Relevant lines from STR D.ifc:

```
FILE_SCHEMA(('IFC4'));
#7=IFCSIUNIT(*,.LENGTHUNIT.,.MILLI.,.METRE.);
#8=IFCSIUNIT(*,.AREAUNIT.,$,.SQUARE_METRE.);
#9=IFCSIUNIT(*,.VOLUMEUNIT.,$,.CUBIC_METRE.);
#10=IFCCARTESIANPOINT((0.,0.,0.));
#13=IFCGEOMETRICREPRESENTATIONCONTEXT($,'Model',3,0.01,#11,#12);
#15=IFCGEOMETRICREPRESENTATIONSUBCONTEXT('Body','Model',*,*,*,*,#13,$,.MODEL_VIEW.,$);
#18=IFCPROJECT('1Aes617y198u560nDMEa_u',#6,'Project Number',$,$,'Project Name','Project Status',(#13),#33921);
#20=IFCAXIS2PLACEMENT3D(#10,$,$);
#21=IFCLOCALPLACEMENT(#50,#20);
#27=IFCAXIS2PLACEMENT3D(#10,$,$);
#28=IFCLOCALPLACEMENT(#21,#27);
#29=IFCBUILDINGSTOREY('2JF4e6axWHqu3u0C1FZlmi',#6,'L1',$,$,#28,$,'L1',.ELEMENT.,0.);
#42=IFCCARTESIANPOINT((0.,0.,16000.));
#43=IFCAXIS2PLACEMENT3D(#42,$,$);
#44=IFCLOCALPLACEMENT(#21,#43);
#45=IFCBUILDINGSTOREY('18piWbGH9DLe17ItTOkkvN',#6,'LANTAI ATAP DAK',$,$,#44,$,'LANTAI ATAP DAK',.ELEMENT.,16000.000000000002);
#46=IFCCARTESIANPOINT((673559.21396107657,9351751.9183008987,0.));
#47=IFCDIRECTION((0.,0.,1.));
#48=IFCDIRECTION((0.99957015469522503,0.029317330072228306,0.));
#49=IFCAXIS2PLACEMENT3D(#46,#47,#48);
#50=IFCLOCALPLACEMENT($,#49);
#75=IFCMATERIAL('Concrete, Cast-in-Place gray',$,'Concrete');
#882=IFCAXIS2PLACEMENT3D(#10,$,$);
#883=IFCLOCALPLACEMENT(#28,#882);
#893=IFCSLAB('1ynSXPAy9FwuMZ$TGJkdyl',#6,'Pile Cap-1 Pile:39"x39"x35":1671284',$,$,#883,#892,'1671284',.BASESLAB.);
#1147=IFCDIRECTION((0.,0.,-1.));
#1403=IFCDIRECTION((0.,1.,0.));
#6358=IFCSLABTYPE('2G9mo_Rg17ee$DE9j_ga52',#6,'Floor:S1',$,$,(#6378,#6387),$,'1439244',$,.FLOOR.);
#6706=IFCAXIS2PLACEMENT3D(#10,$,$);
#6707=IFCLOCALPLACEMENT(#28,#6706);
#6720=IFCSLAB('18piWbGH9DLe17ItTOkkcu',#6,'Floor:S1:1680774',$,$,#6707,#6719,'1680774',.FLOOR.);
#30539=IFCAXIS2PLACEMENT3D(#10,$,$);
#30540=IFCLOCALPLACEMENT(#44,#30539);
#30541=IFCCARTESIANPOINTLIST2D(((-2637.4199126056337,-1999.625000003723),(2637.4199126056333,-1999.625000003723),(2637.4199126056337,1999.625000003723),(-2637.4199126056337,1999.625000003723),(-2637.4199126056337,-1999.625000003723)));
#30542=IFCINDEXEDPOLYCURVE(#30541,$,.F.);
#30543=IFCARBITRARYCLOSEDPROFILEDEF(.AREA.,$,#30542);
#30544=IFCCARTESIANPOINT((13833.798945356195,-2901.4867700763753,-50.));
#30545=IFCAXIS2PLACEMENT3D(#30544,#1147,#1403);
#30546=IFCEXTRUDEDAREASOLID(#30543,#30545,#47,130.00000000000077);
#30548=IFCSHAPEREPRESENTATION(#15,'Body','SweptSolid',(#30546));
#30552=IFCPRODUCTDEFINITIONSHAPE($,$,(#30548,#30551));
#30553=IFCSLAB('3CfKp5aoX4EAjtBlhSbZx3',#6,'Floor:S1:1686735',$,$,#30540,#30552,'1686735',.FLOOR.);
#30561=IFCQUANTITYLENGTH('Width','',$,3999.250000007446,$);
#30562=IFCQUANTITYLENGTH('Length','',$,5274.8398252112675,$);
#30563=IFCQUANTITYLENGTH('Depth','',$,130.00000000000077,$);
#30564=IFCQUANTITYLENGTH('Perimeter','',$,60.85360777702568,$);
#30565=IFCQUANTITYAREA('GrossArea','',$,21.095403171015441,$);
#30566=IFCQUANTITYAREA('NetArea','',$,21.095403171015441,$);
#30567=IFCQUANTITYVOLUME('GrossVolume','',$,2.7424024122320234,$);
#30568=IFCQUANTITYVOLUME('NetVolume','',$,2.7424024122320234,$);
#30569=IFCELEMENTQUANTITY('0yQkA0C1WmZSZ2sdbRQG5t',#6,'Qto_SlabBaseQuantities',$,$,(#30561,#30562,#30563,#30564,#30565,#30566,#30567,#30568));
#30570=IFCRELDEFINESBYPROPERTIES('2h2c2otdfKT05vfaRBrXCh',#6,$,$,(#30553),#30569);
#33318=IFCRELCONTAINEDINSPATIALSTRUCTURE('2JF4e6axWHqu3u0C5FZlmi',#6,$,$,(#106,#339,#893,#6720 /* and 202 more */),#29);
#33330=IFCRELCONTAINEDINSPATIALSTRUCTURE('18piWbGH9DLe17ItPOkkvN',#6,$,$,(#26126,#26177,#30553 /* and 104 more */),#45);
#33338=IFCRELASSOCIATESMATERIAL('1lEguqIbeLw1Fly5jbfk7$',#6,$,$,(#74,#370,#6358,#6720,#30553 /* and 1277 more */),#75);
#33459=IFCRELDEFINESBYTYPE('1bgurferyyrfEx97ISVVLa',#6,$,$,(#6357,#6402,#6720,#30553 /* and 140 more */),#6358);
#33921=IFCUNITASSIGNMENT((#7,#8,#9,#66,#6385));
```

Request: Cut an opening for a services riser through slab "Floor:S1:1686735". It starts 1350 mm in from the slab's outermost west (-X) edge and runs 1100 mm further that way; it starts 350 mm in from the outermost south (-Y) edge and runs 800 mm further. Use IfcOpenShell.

```python
import numpy as np
import ifcopenshell
import ifcopenshell.api.feature
import ifcopenshell.api.geometry
import ifcopenshell.api.pset
import ifcopenshell.api.root
import ifcopenshell.geom
import ifcopenshell.util.element
import ifcopenshell.util.placement
import ifcopenshell.util.representation
import ifcopenshell.util.shape
import ifcopenshell.util.unit

model = ifcopenshell.open("STR D.ifc")
unit_scale = ifcopenshell.util.unit.calculate_unit_scale(model)
area_scale = ifcopenshell.util.unit.calculate_unit_scale(model, "AREAUNIT")
volume_scale = ifcopenshell.util.unit.calculate_unit_scale(model, "VOLUMEUNIT")
settings = ifcopenshell.geom.settings()


def volume(element):
    """Net volume in cubic metres, openings subtracted."""
    shape = ifcopenshell.geom.create_shape(settings, element)
    return ifcopenshell.util.shape.get_volume(shape.geometry)


slab = model.by_guid("3CfKp5aoX4EAjtBlhSbZx3")
before = volume(slab)

# Extent in the slab's own axes, in metres. The edges named are its -X and -Y sides.
slab_shape = ifcopenshell.geom.create_shape(settings, slab)
vertices = ifcopenshell.util.shape.get_vertices(slab_shape.geometry)
x_min, y_min, bottom = vertices.min(axis=0)
top = vertices[:, 2].max()

opening = ifcopenshell.api.root.create_entity(model, ifc_class="IfcOpeningElement", name="Services riser opening", predefined_type="OPENING")
context = ifcopenshell.util.representation.get_context(model, "Model", "Body", "MODEL_VIEW")
width, depth = 1.1, 0.8
outline = [(0.0, 0.0), (width, 0.0), (width, depth), (0.0, depth), (0.0, 0.0)]
# Overshoot both faces by 50 mm so the cut is clean.
shape = ifcopenshell.api.geometry.add_slab_representation(
    model, context=context, depth=top - bottom + 0.1, polyline=outline
)
ifcopenshell.api.geometry.assign_representation(model, product=opening, representation=shape)

matrix = ifcopenshell.util.placement.get_local_placement(slab.ObjectPlacement)
matrix[:, 3] = matrix @ np.append(np.array([x_min + 1.35, y_min + 0.35, bottom - 0.05]) / unit_scale, 1.0)
ifcopenshell.api.geometry.edit_object_placement(model, product=opening, matrix=matrix, is_si=False)
ifcopenshell.api.feature.add_feature(model, feature=opening, element=slab)

after = volume(slab)

# Update the slab's stored quantities.
qto = model.by_id(ifcopenshell.util.element.get_pset(slab, "Qto_SlabBaseQuantities", should_inherit=False)["id"])
ifcopenshell.api.pset.edit_qto(model, qto=qto, properties={
    "NetArea": after / (top - bottom) / area_scale,
    "NetVolume": after / volume_scale,
})

print(f"slab volume {before:.3f} -> {after:.3f} m3")

model.write("STR D-out.ifc")
```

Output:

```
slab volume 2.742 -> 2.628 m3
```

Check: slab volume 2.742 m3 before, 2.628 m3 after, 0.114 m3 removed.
